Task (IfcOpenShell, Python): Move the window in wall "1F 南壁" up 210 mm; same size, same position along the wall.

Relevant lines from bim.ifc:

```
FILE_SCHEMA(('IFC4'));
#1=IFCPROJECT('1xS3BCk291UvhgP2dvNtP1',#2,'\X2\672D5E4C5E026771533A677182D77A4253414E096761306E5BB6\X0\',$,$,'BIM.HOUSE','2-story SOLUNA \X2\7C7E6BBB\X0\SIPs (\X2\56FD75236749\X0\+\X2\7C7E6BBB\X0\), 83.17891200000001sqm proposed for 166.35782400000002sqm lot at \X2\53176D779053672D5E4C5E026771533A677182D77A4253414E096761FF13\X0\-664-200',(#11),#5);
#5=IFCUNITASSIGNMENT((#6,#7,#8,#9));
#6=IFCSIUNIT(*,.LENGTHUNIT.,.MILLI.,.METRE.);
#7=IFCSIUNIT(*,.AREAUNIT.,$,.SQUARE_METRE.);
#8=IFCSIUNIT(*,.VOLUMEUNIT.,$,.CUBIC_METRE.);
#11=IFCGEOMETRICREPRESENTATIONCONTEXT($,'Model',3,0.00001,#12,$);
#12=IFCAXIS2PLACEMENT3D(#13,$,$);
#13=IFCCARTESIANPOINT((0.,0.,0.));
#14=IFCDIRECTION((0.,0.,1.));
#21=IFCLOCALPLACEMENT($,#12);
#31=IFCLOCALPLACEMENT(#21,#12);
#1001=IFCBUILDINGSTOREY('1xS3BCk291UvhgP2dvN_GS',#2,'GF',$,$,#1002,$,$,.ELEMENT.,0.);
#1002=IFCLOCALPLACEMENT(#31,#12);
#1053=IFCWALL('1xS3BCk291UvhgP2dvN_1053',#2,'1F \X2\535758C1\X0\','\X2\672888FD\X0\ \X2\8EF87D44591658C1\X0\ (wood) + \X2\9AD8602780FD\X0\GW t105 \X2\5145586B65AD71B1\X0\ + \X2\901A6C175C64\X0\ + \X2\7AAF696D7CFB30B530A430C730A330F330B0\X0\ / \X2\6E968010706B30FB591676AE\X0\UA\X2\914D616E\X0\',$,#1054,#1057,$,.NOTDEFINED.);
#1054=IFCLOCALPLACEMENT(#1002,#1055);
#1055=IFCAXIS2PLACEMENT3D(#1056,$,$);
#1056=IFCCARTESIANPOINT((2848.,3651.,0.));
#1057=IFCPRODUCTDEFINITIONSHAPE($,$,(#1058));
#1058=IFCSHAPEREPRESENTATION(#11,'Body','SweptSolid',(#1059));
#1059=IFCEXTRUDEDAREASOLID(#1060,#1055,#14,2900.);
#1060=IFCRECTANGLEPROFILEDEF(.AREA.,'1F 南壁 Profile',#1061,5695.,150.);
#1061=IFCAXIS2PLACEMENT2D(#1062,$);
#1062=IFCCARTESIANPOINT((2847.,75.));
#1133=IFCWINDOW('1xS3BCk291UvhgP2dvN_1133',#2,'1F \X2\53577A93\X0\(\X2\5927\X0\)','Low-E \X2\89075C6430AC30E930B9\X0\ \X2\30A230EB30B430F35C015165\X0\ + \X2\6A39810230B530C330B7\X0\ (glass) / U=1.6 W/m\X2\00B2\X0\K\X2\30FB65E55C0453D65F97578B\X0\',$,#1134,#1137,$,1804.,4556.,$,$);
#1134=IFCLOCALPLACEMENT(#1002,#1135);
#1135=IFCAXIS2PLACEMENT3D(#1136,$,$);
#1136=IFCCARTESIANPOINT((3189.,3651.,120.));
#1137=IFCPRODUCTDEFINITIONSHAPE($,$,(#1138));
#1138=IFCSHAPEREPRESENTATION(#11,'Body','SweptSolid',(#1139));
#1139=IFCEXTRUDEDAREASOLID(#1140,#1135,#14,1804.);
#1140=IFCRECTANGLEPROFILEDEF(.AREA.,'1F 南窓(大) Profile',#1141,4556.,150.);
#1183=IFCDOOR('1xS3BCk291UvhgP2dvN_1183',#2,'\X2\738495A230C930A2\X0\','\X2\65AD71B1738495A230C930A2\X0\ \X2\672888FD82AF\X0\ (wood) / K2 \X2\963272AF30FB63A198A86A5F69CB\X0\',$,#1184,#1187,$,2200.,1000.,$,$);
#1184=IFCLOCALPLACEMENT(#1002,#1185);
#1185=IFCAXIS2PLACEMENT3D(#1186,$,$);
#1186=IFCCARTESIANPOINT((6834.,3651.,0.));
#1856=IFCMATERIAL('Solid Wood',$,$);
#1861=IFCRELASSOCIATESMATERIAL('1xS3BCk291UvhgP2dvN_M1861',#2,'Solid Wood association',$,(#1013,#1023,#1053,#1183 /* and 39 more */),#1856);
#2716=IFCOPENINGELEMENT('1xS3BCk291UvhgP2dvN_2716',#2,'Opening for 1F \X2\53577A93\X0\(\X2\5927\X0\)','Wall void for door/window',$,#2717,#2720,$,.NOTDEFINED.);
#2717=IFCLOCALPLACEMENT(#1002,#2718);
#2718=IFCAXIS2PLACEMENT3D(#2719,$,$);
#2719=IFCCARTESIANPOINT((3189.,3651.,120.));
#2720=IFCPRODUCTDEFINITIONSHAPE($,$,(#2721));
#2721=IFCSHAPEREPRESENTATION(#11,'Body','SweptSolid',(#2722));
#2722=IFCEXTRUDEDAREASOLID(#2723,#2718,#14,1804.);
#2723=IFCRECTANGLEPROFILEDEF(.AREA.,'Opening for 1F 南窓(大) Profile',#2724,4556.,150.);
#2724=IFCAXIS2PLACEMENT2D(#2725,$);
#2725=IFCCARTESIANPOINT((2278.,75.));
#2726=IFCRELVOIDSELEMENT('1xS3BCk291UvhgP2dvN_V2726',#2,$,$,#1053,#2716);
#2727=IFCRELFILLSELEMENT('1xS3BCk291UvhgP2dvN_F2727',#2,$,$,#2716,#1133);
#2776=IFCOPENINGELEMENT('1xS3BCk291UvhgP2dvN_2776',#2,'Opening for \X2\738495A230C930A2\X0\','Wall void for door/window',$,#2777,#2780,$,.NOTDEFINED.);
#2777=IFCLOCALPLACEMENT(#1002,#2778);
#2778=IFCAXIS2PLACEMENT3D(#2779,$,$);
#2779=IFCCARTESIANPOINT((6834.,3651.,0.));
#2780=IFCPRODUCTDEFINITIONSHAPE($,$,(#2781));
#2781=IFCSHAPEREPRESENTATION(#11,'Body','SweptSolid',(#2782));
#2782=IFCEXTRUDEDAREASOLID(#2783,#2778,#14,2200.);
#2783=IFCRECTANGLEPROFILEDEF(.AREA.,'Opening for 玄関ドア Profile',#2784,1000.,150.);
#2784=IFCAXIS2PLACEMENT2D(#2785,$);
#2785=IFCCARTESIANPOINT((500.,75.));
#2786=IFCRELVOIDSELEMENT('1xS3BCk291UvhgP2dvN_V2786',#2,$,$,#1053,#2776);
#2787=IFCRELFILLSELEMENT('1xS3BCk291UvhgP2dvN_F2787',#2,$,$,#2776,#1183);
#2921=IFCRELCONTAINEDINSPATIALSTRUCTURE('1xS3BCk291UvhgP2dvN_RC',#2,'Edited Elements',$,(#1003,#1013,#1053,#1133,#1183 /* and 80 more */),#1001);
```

```python
import numpy as np
import ifcopenshell
import ifcopenshell.api.geometry
import ifcopenshell.util.placement
import ifcopenshell.util.unit

model = ifcopenshell.open("bim.ifc")
unit_scale = ifcopenshell.util.unit.calculate_unit_scale(model)

window = model.by_guid("1xS3BCk291UvhgP2dvN_1133")
opening = window.FillsVoids[0].RelatingOpeningElement
dz = 210.0

shift = np.array([0.0, 0.0, dz])
# The window is not placed relative to its opening, so move both.
for product in (opening, window):
    matrix = ifcopenshell.util.placement.get_local_placement(product.ObjectPlacement)
    matrix[:3, 3] += shift
    ifcopenshell.api.geometry.edit_object_placement(model, product=product, matrix=matrix, is_si=False)

print(f"moved by {dz * unit_scale:+.3f} m")

model.write("bim_updated.ifc")
```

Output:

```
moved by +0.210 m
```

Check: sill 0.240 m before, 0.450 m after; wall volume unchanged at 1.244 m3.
